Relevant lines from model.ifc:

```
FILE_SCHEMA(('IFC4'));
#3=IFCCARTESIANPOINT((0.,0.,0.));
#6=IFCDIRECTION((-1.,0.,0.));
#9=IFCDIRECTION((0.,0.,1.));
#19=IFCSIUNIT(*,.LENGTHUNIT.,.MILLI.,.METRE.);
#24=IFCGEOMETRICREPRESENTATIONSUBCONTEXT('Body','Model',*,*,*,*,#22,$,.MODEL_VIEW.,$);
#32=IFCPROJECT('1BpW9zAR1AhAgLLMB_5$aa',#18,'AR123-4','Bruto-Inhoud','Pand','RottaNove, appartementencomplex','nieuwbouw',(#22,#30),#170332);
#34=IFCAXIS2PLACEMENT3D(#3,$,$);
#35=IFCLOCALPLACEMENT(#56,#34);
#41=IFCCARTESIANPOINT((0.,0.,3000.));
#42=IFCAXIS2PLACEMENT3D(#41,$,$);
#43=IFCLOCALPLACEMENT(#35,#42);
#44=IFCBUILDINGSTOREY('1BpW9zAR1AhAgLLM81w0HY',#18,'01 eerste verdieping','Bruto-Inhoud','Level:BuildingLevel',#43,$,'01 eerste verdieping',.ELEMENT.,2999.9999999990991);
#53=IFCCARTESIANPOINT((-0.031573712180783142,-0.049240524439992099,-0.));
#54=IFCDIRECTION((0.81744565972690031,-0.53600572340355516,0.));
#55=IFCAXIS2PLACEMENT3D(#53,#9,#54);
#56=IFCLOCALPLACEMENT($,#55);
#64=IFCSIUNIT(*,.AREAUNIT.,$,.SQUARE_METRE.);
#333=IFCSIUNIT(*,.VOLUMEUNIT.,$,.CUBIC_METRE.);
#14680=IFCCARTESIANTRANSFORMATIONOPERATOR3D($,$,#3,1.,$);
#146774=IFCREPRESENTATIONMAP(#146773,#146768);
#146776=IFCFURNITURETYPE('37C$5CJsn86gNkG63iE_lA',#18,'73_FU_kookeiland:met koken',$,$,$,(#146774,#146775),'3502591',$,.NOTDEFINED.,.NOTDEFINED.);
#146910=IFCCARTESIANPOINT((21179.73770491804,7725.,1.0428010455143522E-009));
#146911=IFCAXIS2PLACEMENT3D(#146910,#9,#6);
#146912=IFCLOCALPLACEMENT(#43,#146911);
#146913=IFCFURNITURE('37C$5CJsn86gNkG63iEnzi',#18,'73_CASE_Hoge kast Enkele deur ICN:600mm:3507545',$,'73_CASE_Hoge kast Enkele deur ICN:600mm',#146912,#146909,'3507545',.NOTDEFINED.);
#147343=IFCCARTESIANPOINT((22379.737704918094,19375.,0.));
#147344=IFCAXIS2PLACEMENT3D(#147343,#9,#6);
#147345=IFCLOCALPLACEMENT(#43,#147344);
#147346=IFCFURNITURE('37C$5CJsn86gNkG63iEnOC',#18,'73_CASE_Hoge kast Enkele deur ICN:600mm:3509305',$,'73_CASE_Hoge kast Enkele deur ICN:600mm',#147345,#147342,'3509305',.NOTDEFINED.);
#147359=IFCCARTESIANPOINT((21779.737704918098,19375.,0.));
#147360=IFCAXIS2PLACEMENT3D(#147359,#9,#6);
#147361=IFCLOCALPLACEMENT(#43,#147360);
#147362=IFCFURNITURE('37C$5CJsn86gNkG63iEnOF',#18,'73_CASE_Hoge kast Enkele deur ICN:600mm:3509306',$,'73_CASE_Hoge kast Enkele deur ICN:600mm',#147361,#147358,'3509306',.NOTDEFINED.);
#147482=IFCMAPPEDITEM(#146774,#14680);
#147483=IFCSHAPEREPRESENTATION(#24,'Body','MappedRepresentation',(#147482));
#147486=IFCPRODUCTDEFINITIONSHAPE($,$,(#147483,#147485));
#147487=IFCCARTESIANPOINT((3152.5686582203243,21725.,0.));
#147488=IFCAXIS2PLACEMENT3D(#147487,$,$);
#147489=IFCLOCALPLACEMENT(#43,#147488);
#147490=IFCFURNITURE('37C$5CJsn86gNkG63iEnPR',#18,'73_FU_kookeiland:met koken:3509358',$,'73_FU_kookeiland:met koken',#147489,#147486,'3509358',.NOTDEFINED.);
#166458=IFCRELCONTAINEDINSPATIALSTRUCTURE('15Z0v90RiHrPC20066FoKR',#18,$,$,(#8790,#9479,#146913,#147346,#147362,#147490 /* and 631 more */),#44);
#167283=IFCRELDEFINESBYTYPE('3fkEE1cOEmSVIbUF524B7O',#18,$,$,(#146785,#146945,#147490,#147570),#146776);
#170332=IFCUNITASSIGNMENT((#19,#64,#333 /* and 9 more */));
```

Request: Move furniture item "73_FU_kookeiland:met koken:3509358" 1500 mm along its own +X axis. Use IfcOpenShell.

```python
import ifcopenshell
import ifcopenshell.api.geometry
import ifcopenshell.util.placement

model = ifcopenshell.open("model.ifc")

item = model.by_id(147490)
matrix = ifcopenshell.util.placement.get_local_placement(item.ObjectPlacement)
matrix[:3, 3] += matrix[:3, 0] * 1500.0
ifcopenshell.api.geometry.edit_object_placement(model, product=item, matrix=matrix, is_si=False)

print(ifcopenshell.util.placement.get_local_placement(item.ObjectPlacement).round(3) + 0.0)

model.write("model_edited.ifc")
```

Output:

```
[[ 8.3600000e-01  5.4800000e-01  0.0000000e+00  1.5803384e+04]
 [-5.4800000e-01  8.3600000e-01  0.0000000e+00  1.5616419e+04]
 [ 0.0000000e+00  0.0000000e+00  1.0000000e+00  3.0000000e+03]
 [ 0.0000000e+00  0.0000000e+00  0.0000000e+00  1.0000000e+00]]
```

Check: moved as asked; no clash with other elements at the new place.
